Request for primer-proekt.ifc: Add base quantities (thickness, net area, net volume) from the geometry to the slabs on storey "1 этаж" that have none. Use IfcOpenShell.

First a look at what the model holds.

```python
import ifcopenshell
import ifcopenshell.util.element
import ifcopenshell.util.unit

model = ifcopenshell.open("primer-proekt.ifc")
print(model.schema)
for unit_type in ("LENGTHUNIT", "AREAUNIT", "VOLUMEUNIT"):
    print(unit_type, ifcopenshell.util.unit.calculate_unit_scale(model, unit_type))
storey = next(s for s in model.by_type("IfcBuildingStorey") if s.Name == "1 этаж")
slabs = [e for e in ifcopenshell.util.element.get_decomposition(storey) if e.is_a("IfcSlab")]
for e in sorted(slabs, key=lambda e: e.id()):
    print(e.id(), e.is_a(), e.Name, list(ifcopenshell.util.element.get_psets(e, qtos_only=True)), sep=" | ")
```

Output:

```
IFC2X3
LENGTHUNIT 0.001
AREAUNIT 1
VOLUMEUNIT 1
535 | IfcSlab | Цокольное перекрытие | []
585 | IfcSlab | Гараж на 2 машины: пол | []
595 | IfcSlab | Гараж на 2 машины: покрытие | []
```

```python
import ifcopenshell
import ifcopenshell.api.pset
import ifcopenshell.geom
import ifcopenshell.util.element
import ifcopenshell.util.shape
import ifcopenshell.util.unit

model = ifcopenshell.open("primer-proekt.ifc")
unit_scale = ifcopenshell.util.unit.calculate_unit_scale(model)
area_scale = ifcopenshell.util.unit.calculate_unit_scale(model, "AREAUNIT")
volume_scale = ifcopenshell.util.unit.calculate_unit_scale(model, "VOLUMEUNIT")
settings = ifcopenshell.geom.settings()

storey = next(s for s in model.by_type("IfcBuildingStorey") if s.Name == "1 этаж")
slabs = [e for e in ifcopenshell.util.element.get_decomposition(storey) if e.is_a("IfcSlab")]

for e in sorted(slabs, key=lambda e: e.id()):
    if ifcopenshell.util.element.get_psets(e, qtos_only=True, should_inherit=False):
        continue
    # Geometry comes back in metres, in the element's own axes.
    shape = ifcopenshell.geom.create_shape(settings, e)
    values = {
        "Width": ifcopenshell.util.shape.get_z(shape.geometry) / unit_scale,
        "NetArea": ifcopenshell.util.shape.get_footprint_area(shape.geometry) / area_scale,
        "NetVolume": ifcopenshell.util.shape.get_volume(shape.geometry) / volume_scale,
    }
    qto = ifcopenshell.api.pset.add_qto(model, product=e, name="BaseQuantities")
    ifcopenshell.api.pset.edit_qto(model, qto=qto, properties=values)
    print(e.id(), {k: round(v, 3) for k, v in values.items()})

model.write("primer-proekt_v2.ifc")
```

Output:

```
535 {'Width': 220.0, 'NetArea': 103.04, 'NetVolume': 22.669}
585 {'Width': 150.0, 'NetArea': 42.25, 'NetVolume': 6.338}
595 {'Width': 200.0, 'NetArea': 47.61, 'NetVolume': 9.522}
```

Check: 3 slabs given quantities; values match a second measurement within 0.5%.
